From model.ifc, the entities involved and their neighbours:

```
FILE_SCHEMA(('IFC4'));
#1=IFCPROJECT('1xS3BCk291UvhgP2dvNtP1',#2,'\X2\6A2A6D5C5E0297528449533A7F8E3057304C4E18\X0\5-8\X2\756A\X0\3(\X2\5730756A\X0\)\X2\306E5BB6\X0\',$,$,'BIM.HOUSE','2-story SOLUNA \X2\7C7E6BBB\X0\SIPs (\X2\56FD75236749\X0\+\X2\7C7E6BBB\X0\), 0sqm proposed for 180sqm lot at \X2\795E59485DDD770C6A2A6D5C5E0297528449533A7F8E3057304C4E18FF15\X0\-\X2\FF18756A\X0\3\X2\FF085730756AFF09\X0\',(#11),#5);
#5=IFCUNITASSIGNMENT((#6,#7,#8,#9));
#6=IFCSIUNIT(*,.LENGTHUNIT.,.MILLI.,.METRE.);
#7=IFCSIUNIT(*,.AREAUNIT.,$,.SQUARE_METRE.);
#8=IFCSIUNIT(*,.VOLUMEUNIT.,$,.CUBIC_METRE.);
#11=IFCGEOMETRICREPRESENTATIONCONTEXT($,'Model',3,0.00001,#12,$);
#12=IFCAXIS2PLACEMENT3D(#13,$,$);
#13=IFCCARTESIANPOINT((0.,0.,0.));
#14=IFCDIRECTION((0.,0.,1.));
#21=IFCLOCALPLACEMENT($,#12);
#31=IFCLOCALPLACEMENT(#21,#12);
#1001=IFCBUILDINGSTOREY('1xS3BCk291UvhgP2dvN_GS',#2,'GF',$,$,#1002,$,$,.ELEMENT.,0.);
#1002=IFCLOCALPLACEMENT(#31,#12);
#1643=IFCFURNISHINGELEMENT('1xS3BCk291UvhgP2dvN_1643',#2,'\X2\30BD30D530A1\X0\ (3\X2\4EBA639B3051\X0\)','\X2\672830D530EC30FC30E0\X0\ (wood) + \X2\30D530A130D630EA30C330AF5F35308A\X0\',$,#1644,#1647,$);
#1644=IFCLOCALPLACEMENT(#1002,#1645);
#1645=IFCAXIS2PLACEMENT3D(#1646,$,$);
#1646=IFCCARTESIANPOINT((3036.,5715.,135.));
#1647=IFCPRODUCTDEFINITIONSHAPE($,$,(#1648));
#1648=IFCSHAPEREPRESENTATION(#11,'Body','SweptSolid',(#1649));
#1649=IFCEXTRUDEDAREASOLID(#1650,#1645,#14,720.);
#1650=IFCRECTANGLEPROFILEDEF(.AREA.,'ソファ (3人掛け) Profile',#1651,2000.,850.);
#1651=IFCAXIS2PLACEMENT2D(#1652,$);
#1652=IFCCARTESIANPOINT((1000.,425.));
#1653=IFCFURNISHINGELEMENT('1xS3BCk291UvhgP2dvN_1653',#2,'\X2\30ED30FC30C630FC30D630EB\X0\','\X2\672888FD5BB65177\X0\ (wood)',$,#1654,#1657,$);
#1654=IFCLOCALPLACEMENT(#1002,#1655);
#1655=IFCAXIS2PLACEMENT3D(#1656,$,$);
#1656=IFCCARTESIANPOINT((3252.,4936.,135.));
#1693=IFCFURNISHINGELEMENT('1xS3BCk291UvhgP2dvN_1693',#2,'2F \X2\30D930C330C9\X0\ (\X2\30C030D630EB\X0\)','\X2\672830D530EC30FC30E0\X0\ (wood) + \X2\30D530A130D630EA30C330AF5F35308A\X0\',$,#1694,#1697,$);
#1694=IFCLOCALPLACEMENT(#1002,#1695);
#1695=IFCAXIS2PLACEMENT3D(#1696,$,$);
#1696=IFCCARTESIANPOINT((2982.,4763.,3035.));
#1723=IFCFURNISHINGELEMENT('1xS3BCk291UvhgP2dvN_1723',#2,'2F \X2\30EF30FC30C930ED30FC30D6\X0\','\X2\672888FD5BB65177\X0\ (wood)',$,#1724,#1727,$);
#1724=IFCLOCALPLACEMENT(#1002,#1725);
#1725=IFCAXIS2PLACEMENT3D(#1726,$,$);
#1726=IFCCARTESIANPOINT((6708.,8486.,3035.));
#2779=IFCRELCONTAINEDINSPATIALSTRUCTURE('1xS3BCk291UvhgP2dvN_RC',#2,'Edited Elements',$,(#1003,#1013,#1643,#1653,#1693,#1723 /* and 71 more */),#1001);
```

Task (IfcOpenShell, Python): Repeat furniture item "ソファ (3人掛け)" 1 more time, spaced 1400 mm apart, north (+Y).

```python
import numpy as np
import ifcopenshell
import ifcopenshell.api.geometry
import ifcopenshell.api.root
import ifcopenshell.util.element
import ifcopenshell.util.placement
import ifcopenshell.util.unit

model = ifcopenshell.open("model.ifc")
unit_scale = ifcopenshell.util.unit.calculate_unit_scale(model)


def reuse_history(source, copy):
    """copy_class also copies each property set's owner history, people and application; keep the originals."""
    for rel in copy.IsDefinedBy:
        if rel.is_a("IfcRelDefinesByProperties") and (history := rel.RelatingPropertyDefinition.OwnerHistory):
            rel.RelatingPropertyDefinition.OwnerHistory = source.OwnerHistory
            ifcopenshell.util.element.remove_deep2(model, history)


source = model.by_guid("1xS3BCk291UvhgP2dvN_1643")
base = ifcopenshell.util.placement.get_local_placement(source.ObjectPlacement)
step = np.array([0.0, 1.0, 0.0]) * 1.4 / unit_scale

for i in range(1, 2):
    copy = ifcopenshell.api.root.copy_class(model, product=source)
    copy.Representation = ifcopenshell.util.element.copy_deep(
        model, source.Representation, exclude=["IfcGeometricRepresentationContext", "IfcRepresentationMap"]
    )
    reuse_history(source, copy)
    matrix = base.copy()
    matrix[:3, 3] += i * step
    print("added at", matrix[:3, 3].round(3) + 0.0)
    ifcopenshell.api.geometry.edit_object_placement(model, product=copy, matrix=matrix, is_si=False)

model.write("model_updated.ifc")
```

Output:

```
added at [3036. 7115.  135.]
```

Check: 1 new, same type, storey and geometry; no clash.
